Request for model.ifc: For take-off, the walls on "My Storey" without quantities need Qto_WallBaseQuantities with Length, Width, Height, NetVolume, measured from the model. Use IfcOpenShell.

First a look at what the model holds.

```python
import ifcopenshell
import ifcopenshell.util.element
import ifcopenshell.util.unit

model = ifcopenshell.open("model.ifc")
print(model.schema)
for unit_type in ("LENGTHUNIT", "AREAUNIT", "VOLUMEUNIT"):
    print(unit_type, ifcopenshell.util.unit.calculate_unit_scale(model, unit_type))
storey = next(s for s in model.by_type("IfcBuildingStorey") if s.Name == "My Storey")
walls = [e for e in ifcopenshell.util.element.get_decomposition(storey) if e.is_a("IfcWall")]
for e in sorted(walls, key=lambda e: e.id()):
    print(e.id(), e.is_a(), e.Name, list(ifcopenshell.util.element.get_psets(e, qtos_only=True)), sep=" | ")
```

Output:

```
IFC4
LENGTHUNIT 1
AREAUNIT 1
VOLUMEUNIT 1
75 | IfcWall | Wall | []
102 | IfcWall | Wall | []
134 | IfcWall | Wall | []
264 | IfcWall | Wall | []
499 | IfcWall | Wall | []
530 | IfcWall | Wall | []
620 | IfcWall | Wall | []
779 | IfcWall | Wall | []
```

```python
import ifcopenshell
import ifcopenshell.api.pset
import ifcopenshell.geom
import ifcopenshell.util.element
import ifcopenshell.util.shape
import ifcopenshell.util.unit

model = ifcopenshell.open("model.ifc")
unit_scale = ifcopenshell.util.unit.calculate_unit_scale(model)
volume_scale = ifcopenshell.util.unit.calculate_unit_scale(model, "VOLUMEUNIT")
settings = ifcopenshell.geom.settings()

storey = next(s for s in model.by_type("IfcBuildingStorey") if s.Name == "My Storey")
walls = [e for e in ifcopenshell.util.element.get_decomposition(storey) if e.is_a("IfcWall")]

for e in sorted(walls, key=lambda e: e.id()):
    if ifcopenshell.util.element.get_psets(e, qtos_only=True, should_inherit=False):
        continue
    # Geometry comes back in metres, in the element's own axes.
    shape = ifcopenshell.geom.create_shape(settings, e)
    values = {
        "Length": ifcopenshell.util.shape.get_x(shape.geometry) / unit_scale,
        "Width": ifcopenshell.util.shape.get_y(shape.geometry) / unit_scale,
        "Height": ifcopenshell.util.shape.get_z(shape.geometry) / unit_scale,
        "NetVolume": ifcopenshell.util.shape.get_volume(shape.geometry) / volume_scale,
    }
    qto = ifcopenshell.api.pset.add_qto(model, product=e, name="Qto_WallBaseQuantities")
    ifcopenshell.api.pset.edit_qto(model, qto=qto, properties=values)
    print(e.id(), {k: round(v, 3) for k, v in values.items()})

model.write("model_updated.ifc")
```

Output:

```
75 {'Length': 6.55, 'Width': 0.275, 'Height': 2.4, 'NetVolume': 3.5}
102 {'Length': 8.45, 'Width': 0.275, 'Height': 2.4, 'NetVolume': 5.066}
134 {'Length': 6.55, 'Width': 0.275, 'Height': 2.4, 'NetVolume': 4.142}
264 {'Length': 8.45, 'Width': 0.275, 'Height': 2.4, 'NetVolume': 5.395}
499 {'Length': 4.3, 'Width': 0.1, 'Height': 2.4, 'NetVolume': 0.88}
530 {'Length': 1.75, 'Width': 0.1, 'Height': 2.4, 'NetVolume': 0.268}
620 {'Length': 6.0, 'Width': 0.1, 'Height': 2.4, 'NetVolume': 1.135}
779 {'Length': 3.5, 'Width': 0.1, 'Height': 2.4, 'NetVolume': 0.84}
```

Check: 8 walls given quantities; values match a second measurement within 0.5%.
